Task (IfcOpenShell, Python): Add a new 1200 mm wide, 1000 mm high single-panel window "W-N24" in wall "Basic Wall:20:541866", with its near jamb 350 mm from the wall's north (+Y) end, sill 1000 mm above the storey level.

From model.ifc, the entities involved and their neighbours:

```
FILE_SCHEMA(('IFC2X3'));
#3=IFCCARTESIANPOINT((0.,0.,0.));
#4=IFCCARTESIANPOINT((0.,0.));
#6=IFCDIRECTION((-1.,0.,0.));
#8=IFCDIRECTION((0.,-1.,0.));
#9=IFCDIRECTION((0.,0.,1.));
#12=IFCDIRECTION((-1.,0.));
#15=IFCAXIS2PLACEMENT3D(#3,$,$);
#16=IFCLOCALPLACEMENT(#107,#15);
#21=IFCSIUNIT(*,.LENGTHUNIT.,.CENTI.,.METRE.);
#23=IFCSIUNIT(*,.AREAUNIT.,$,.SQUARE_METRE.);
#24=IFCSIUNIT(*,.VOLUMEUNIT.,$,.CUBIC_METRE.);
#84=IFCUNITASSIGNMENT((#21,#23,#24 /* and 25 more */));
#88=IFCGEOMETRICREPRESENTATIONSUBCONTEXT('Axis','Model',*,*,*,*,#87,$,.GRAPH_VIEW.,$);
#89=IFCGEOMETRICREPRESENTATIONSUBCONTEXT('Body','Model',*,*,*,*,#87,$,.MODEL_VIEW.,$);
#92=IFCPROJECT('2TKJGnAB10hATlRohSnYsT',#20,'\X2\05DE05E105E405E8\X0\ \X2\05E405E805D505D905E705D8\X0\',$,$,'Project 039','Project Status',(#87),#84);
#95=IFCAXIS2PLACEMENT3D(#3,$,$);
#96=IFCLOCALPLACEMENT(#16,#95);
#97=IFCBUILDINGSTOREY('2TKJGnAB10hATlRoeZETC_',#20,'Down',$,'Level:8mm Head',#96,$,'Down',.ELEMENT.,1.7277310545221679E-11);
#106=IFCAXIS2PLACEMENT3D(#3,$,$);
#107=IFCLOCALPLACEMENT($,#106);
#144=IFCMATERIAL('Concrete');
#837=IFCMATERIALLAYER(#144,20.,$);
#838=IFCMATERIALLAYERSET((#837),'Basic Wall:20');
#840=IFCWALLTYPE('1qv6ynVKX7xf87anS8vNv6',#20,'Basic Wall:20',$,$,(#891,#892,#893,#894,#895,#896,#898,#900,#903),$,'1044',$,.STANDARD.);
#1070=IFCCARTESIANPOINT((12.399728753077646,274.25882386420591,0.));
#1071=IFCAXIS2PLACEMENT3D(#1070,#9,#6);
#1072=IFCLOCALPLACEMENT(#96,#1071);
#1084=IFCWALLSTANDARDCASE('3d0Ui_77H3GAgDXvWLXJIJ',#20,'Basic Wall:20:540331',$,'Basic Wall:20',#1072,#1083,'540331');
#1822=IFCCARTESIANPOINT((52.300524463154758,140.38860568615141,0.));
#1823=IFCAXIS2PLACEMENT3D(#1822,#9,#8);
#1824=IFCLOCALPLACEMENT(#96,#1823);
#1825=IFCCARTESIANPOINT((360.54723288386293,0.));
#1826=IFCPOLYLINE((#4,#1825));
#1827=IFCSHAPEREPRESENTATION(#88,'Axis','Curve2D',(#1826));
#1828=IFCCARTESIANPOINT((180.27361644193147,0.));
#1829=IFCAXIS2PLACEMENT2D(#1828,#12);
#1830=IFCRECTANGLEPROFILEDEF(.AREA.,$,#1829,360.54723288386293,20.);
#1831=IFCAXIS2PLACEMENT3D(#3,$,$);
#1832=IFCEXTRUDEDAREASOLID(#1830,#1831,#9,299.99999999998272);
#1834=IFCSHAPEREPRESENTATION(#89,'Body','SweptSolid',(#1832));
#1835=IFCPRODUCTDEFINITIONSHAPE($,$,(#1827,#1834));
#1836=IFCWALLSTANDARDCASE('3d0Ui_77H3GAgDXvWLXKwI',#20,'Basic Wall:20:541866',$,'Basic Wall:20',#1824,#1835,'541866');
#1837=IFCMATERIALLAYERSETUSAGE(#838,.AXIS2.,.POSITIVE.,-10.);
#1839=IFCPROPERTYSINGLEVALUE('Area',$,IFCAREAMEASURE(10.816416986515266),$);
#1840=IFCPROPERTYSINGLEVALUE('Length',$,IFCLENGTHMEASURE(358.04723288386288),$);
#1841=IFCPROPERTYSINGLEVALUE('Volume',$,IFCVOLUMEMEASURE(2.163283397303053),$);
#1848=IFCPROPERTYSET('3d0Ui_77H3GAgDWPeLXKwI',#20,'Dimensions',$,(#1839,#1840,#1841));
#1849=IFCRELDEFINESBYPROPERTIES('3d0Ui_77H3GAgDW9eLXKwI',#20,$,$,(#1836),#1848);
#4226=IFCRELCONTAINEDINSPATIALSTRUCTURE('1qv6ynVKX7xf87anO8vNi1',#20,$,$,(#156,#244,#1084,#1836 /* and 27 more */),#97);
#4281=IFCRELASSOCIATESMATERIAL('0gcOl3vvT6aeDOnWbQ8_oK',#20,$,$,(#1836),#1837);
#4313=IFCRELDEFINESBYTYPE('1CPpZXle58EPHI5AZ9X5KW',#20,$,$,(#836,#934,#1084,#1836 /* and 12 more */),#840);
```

```python
import numpy as np
import ifcopenshell
import ifcopenshell.api.feature
import ifcopenshell.api.geometry
import ifcopenshell.api.pset
import ifcopenshell.api.root
import ifcopenshell.api.spatial
import ifcopenshell.api.type
import ifcopenshell.geom
import ifcopenshell.util.element
import ifcopenshell.util.placement
import ifcopenshell.util.representation
import ifcopenshell.util.shape
import ifcopenshell.util.unit

model = ifcopenshell.open("model.ifc")
unit_scale = ifcopenshell.util.unit.calculate_unit_scale(model)
area_scale = ifcopenshell.util.unit.calculate_unit_scale(model, "AREAUNIT")
volume_scale = ifcopenshell.util.unit.calculate_unit_scale(model, "VOLUMEUNIT")
settings = ifcopenshell.geom.settings()


def volume(element):
    """Net volume in cubic metres, openings subtracted."""
    shape = ifcopenshell.geom.create_shape(settings, element)
    return ifcopenshell.util.shape.get_volume(shape.geometry)


wall = model.by_guid("3d0Ui_77H3GAgDXvWLXKwI")
storey = ifcopenshell.util.element.get_container(wall, ifc_class="IfcBuildingStorey")
context = ifcopenshell.util.representation.get_context(model, "Model", "Body", "MODEL_VIEW")
before = volume(wall)

width, height, from_end, sill = 1.2, 1, 0.35, 1  # metres

# The wall runs along its own X axis, and the end named is its -X end.
wall_shape = ifcopenshell.geom.create_shape(settings, wall)
x, y, z = ifcopenshell.util.shape.get_vertices(wall_shape.geometry).T
start = x.min() + from_end
face, thickness = float(y.min()), float(y.max() - y.min())
wall_matrix = ifcopenshell.util.placement.get_local_placement(wall.ObjectPlacement)
level = ifcopenshell.util.placement.get_local_placement(storey.ObjectPlacement)[2, 3]


def in_wall(x, y):
    """Placement at x, y metres in the wall's axes, at sill height."""
    matrix = wall_matrix.copy()
    matrix[:, 3] = wall_matrix @ np.array([x / unit_scale, y / unit_scale, 0.0, 1.0])
    matrix[2, 3] = level + sill / unit_scale
    return matrix


# Opening: a box that overshoots both wall faces by 50 mm.
opening = ifcopenshell.api.root.create_entity(model, ifc_class="IfcOpeningElement")
box = ifcopenshell.api.geometry.add_wall_representation(
    model, context=context, length=width, height=height, thickness=thickness + 0.1
)
ifcopenshell.api.geometry.assign_representation(model, product=opening, representation=box)
ifcopenshell.api.geometry.edit_object_placement(model, product=opening, matrix=in_wall(start, face - 0.05), is_si=False)
ifcopenshell.api.feature.add_feature(model, feature=opening, element=wall)

window = ifcopenshell.api.root.create_entity(model, ifc_class="IfcWindow", name="W-N24")
window.OverallWidth, window.OverallHeight = width / unit_scale, height / unit_scale
body = ifcopenshell.api.geometry.add_window_representation(
    model,
    context=context,
    overall_width=window.OverallWidth,
    overall_height=window.OverallHeight,
    partition_type="SINGLE_PANEL",
)
ifcopenshell.api.geometry.assign_representation(model, product=window, representation=body)
ifcopenshell.api.spatial.assign_container(model, products=[window], relating_structure=storey)
fills = ifcopenshell.api.feature.add_filling(model, opening=opening, element=window)
fills.OwnerHistory = window.OwnerHistory  # required in IFC2X3

# IFC2X3 keeps the operation on the window style.
style = ifcopenshell.api.root.create_entity(model, ifc_class="IfcWindowStyle", name="W-N24")
style.OperationType, style.ConstructionType = "SINGLE_PANEL", "NOTDEFINED"
style.ParameterTakesPrecedence = style.Sizeable = False
ifcopenshell.api.type.assign_type(model, related_objects=[window], relating_type=style)

# Centre the window in the wall's thickness.
ifcopenshell.api.geometry.edit_object_placement(model, product=window, matrix=in_wall(start, face), is_si=False)
window_shape = ifcopenshell.geom.create_shape(settings, window)
depth = ifcopenshell.util.shape.get_vertices(window_shape.geometry)[:, 1]
offset = face + thickness / 2 - (depth.min() + depth.max()) / 2
ifcopenshell.api.geometry.edit_object_placement(model, product=window, matrix=in_wall(start, offset), is_si=False)

after = volume(wall)

# Update the wall's stored quantities.
pset = model.by_id(ifcopenshell.util.element.get_pset(wall, "Dimensions", should_inherit=False)["id"])
ifcopenshell.api.pset.edit_pset(model, pset=pset, properties={
    "Area": model.create_entity("IfcAreaMeasure", after / thickness / area_scale),
    "Volume": model.create_entity("IfcVolumeMeasure", after / volume_scale),
})

print(f"wall volume {before:.3f} -> {after:.3f} m3")

model.write("model-out.ifc")
```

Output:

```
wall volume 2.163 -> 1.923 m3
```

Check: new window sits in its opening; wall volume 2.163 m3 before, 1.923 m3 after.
